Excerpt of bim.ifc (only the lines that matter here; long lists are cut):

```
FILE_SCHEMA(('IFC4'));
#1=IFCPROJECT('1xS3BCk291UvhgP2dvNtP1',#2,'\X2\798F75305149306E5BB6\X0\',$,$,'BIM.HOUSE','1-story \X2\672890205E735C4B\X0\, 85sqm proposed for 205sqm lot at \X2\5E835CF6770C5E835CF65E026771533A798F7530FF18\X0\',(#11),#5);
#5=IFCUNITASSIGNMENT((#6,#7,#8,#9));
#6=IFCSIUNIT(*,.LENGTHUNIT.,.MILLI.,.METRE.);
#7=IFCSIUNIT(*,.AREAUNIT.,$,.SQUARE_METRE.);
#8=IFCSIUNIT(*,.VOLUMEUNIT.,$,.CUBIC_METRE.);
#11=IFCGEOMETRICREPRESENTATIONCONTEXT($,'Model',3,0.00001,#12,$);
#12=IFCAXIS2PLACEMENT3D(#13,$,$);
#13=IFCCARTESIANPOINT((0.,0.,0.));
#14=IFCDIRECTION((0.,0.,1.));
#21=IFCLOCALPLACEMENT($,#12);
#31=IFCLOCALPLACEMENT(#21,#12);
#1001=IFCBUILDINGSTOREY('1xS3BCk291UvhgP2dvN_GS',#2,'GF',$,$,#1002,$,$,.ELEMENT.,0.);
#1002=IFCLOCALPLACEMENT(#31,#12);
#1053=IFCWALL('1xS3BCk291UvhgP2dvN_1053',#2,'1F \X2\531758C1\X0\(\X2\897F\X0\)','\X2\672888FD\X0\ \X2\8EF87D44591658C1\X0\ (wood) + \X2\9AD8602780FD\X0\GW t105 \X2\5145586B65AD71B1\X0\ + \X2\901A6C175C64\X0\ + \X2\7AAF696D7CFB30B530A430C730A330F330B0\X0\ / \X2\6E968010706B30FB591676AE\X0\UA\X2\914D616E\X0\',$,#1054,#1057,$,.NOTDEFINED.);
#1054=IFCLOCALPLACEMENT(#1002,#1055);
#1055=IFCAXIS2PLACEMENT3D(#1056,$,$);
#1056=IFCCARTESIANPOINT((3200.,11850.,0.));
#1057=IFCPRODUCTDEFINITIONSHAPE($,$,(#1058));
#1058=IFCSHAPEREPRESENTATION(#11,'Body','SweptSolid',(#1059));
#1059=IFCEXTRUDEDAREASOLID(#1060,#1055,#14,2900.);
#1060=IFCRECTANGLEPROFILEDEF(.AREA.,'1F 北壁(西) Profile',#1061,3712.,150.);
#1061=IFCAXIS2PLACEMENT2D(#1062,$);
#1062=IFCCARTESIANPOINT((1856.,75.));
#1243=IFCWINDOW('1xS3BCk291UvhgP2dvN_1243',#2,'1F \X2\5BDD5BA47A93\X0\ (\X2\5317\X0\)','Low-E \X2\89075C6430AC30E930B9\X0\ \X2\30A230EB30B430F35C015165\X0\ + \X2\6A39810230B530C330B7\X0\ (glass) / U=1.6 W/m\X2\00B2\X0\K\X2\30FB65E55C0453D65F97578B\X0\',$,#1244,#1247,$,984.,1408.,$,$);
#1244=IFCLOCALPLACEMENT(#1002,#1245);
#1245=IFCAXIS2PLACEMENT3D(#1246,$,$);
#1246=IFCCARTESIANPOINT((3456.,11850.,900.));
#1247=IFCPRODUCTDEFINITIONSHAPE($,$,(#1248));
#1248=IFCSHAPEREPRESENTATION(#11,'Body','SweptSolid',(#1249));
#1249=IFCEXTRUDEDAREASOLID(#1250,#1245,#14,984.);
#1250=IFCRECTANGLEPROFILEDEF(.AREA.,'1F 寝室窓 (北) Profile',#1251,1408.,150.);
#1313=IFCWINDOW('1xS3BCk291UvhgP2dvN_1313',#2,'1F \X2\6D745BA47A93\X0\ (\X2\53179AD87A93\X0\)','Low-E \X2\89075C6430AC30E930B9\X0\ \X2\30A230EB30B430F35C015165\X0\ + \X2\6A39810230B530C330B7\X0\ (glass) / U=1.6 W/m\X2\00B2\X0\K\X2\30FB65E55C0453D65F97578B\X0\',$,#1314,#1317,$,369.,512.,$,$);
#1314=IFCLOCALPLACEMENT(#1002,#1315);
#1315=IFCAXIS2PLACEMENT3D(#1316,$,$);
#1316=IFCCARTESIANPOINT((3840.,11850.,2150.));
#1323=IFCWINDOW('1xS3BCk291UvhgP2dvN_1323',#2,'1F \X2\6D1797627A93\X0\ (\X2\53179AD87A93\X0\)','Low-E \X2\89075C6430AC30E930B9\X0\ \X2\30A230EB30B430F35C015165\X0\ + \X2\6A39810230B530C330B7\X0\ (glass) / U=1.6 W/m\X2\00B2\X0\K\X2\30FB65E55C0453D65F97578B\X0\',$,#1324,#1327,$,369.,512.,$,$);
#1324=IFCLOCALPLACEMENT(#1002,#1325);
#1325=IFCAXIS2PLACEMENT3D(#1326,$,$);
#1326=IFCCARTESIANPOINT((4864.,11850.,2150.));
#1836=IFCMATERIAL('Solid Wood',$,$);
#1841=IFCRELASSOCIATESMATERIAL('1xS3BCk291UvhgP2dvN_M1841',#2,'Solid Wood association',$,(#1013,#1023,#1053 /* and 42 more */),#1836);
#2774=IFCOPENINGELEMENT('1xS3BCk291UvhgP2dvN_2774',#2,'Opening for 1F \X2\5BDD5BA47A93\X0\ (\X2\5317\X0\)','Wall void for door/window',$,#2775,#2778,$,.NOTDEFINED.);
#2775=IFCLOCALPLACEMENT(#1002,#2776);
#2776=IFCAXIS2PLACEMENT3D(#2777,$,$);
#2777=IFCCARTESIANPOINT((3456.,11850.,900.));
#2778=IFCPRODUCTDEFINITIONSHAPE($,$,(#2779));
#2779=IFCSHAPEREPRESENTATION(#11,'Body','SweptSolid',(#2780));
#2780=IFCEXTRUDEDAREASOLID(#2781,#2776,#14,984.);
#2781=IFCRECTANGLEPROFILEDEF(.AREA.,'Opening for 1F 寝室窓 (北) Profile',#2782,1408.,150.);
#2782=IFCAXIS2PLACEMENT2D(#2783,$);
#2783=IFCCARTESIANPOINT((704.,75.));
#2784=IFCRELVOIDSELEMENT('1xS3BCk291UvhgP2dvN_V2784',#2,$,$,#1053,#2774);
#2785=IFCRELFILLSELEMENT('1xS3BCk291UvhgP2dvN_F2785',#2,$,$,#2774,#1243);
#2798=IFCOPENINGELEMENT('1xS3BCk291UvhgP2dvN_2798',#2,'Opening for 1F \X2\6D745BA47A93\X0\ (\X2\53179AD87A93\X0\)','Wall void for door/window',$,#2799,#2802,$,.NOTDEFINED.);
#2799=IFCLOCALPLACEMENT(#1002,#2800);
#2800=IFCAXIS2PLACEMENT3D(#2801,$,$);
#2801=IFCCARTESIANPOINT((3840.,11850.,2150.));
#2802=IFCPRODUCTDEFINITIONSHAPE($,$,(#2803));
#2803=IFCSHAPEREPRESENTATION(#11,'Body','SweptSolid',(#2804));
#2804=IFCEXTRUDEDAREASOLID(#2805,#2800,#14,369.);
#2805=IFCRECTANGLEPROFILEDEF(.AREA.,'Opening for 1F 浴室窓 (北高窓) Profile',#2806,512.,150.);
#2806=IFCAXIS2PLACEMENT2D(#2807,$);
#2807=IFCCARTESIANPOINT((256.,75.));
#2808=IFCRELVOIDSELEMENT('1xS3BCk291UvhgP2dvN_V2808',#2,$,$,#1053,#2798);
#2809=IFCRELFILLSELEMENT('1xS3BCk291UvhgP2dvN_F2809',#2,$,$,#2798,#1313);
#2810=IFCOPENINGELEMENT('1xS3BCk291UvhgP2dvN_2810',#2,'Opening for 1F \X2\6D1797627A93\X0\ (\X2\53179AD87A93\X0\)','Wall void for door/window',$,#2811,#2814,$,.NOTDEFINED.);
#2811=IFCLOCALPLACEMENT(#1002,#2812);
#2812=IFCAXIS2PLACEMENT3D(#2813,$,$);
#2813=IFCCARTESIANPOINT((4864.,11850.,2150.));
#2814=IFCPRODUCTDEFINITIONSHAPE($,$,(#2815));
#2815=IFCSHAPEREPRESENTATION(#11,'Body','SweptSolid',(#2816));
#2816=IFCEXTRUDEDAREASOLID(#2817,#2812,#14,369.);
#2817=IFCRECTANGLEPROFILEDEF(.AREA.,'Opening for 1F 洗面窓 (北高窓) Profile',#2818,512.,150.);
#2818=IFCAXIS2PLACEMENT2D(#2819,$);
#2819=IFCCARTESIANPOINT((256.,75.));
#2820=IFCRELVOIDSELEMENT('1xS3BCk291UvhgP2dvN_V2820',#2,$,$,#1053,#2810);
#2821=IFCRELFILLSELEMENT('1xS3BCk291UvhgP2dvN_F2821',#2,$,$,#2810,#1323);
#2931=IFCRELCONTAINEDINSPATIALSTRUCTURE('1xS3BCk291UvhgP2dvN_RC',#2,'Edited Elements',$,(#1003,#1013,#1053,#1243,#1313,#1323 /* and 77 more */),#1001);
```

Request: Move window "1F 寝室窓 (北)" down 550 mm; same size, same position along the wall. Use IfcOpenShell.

```python
import numpy as np
import ifcopenshell
import ifcopenshell.api.geometry
import ifcopenshell.util.placement
import ifcopenshell.util.unit

model = ifcopenshell.open("bim.ifc")
unit_scale = ifcopenshell.util.unit.calculate_unit_scale(model)

window = model.by_guid("1xS3BCk291UvhgP2dvN_1243")
opening = window.FillsVoids[0].RelatingOpeningElement
dz = -0.55 / unit_scale

shift = np.array([0.0, 0.0, dz])
# The window is not placed relative to its opening, so move both.
for product in (opening, window):
    matrix = ifcopenshell.util.placement.get_local_placement(product.ObjectPlacement)
    matrix[:3, 3] += shift
    ifcopenshell.api.geometry.edit_object_placement(model, product=product, matrix=matrix, is_si=False)

print(f"moved by {dz * unit_scale:+.3f} m")

model.write("bim_v2.ifc")
```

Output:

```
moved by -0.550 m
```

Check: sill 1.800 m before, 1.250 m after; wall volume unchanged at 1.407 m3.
